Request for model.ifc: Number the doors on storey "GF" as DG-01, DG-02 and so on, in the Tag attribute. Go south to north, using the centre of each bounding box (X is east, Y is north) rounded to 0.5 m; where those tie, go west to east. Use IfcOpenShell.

First a look at what the model holds.

```python
import ifcopenshell
import ifcopenshell.util.element
import ifcopenshell.util.placement

model = ifcopenshell.open("model.ifc")
print(model.schema)
storey = next(s for s in model.by_type("IfcBuildingStorey") if s.Name == "GF")
doors = [e for e in ifcopenshell.util.element.get_decomposition(storey) if e.is_a("IfcDoor")]
for e in sorted(doors, key=lambda e: e.id()):
    origin = ifcopenshell.util.placement.get_local_placement(e.ObjectPlacement)[:3, 3]
    print(e.id(), e.Tag, e.Name, origin.round(2) + 0.0, sep=" | ")
```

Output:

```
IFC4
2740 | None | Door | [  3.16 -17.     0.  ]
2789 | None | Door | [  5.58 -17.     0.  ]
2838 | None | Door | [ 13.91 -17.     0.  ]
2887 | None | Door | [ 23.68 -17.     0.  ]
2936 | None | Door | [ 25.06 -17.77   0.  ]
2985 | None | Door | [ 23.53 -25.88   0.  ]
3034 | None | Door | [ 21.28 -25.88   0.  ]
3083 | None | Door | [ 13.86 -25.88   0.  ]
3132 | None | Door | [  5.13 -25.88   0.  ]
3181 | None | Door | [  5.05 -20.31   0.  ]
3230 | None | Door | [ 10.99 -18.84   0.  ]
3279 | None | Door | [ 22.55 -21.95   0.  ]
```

```python
import ifcopenshell
import ifcopenshell.geom
import ifcopenshell.util.element
import ifcopenshell.util.shape

model = ifcopenshell.open("model.ifc")
settings = ifcopenshell.geom.settings()
settings.set("use-world-coords", True)


def centre(element):
    shape = ifcopenshell.geom.create_shape(settings, element)
    return ifcopenshell.util.shape.get_bbox_centroid(shape.geometry)


storey = next(s for s in model.by_type("IfcBuildingStorey") if s.Name == "GF")
doors = [e for e in ifcopenshell.util.element.get_decomposition(storey) if e.is_a("IfcDoor")]

# Insertion points can sit at a corner or the storey origin, so sort by the geometry (in metres).
centres = {e: centre(e) for e in doors}
doors.sort(key=lambda e: (round(centres[e][1] / 0.5), centres[e][0]))

for i, e in enumerate(doors, start=1):
    number = f"DG-{i:02d}"
    e.Tag = number
    print(e.id(), number)

model.write("model_v2.ifc")
```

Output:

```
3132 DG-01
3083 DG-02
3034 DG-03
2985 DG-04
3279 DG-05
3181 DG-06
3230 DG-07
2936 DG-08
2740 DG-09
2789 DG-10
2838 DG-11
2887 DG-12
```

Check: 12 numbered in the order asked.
